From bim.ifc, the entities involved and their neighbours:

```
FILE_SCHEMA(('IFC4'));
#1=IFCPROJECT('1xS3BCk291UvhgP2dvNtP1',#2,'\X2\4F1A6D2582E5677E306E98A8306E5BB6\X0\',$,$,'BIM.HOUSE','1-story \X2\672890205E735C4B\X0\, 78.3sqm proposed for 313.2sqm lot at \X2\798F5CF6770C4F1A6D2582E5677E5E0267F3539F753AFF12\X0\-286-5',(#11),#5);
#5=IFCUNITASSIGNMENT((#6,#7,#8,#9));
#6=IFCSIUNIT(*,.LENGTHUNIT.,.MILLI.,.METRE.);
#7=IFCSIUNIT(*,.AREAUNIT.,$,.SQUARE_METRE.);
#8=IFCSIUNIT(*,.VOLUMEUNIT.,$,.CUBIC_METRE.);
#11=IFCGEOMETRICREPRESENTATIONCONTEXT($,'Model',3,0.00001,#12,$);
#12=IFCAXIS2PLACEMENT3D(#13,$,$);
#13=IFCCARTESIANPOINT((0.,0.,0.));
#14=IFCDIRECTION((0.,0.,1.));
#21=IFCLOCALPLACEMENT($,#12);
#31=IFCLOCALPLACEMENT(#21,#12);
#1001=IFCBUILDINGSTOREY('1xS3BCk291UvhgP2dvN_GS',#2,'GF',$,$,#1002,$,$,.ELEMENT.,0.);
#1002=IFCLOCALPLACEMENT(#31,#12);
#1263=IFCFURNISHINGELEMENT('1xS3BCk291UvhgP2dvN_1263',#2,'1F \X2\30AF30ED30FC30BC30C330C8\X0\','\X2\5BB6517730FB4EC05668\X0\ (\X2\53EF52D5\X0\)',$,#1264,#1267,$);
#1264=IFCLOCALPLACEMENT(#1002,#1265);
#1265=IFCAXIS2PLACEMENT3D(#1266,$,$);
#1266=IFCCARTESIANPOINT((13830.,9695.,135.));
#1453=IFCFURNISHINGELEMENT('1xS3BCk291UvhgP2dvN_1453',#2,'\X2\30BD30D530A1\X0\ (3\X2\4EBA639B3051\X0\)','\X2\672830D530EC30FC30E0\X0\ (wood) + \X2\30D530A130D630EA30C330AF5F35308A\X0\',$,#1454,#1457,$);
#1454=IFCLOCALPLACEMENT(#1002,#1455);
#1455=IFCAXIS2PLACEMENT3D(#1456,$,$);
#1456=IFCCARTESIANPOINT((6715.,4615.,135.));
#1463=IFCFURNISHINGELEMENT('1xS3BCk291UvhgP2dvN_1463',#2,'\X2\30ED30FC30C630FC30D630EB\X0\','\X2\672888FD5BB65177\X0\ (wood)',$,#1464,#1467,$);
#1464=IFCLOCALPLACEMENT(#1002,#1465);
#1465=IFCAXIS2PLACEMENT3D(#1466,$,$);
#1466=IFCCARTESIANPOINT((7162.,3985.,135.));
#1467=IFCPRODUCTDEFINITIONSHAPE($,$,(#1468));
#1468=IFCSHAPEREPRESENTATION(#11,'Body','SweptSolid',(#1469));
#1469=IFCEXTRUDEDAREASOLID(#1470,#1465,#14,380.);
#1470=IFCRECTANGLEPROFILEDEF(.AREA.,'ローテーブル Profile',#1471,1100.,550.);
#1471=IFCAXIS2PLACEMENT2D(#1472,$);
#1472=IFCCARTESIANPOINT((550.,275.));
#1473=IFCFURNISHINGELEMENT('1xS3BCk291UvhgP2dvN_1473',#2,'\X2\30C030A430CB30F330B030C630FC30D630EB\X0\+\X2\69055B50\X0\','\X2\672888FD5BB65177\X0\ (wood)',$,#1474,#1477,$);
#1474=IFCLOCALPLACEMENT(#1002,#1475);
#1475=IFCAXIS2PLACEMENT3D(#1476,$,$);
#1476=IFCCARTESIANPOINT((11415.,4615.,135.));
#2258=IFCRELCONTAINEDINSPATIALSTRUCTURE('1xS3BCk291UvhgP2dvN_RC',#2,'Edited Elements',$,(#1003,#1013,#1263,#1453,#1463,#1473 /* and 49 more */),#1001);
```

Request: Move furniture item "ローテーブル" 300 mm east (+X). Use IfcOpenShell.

```python
import ifcopenshell
import ifcopenshell.api.geometry
import ifcopenshell.util.placement

model = ifcopenshell.open("bim.ifc")

item = model.by_id(1463)
matrix = ifcopenshell.util.placement.get_local_placement(item.ObjectPlacement)
matrix[0, 3] += 300.0
ifcopenshell.api.geometry.edit_object_placement(model, product=item, matrix=matrix, is_si=False)

print(ifcopenshell.util.placement.get_local_placement(item.ObjectPlacement).round(3) + 0.0)

model.write("bim_rev.ifc")
```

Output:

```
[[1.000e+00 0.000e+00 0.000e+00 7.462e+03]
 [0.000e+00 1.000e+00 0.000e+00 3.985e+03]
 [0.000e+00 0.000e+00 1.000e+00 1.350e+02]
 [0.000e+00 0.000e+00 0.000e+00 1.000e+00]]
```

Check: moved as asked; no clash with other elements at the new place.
